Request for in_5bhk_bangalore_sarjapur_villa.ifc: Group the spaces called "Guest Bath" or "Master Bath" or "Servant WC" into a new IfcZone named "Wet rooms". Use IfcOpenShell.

First a look at what the model holds.

```python
import ifcopenshell

model = ifcopenshell.open("in_5bhk_bangalore_sarjapur_villa.ifc")
print(model.schema)
seen = {}
for space in model.by_type("IfcSpace"):
    seen[space.LongName] = seen.get(space.LongName, 0) + 1
for name, count in sorted(seen.items(), key=str):
    print(count, "x", name)
print("zones:", [z.Name for z in model.by_type("IfcZone")][:20])
```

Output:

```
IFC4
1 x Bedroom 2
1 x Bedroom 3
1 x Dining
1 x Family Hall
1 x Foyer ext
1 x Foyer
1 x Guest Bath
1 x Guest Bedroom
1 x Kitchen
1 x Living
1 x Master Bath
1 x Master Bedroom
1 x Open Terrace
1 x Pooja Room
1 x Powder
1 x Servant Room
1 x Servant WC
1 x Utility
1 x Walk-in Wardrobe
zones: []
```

```python
import ifcopenshell
import ifcopenshell.api.group
import ifcopenshell.api.root

model = ifcopenshell.open("in_5bhk_bangalore_sarjapur_villa.ifc")

names = {"Guest Bath", "Master Bath", "Servant WC"}
spaces = [s for s in model.by_type("IfcSpace") if s.LongName in names]

zone = ifcopenshell.api.root.create_entity(model, ifc_class="IfcZone", name="Wet rooms")
ifcopenshell.api.group.assign_group(model, products=spaces, group=zone)
print(len(spaces), "spaces in", zone.Name)

model.write("in_5bhk_bangalore_sarjapur_villa_edited.ifc")
```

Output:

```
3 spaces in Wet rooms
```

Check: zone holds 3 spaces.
